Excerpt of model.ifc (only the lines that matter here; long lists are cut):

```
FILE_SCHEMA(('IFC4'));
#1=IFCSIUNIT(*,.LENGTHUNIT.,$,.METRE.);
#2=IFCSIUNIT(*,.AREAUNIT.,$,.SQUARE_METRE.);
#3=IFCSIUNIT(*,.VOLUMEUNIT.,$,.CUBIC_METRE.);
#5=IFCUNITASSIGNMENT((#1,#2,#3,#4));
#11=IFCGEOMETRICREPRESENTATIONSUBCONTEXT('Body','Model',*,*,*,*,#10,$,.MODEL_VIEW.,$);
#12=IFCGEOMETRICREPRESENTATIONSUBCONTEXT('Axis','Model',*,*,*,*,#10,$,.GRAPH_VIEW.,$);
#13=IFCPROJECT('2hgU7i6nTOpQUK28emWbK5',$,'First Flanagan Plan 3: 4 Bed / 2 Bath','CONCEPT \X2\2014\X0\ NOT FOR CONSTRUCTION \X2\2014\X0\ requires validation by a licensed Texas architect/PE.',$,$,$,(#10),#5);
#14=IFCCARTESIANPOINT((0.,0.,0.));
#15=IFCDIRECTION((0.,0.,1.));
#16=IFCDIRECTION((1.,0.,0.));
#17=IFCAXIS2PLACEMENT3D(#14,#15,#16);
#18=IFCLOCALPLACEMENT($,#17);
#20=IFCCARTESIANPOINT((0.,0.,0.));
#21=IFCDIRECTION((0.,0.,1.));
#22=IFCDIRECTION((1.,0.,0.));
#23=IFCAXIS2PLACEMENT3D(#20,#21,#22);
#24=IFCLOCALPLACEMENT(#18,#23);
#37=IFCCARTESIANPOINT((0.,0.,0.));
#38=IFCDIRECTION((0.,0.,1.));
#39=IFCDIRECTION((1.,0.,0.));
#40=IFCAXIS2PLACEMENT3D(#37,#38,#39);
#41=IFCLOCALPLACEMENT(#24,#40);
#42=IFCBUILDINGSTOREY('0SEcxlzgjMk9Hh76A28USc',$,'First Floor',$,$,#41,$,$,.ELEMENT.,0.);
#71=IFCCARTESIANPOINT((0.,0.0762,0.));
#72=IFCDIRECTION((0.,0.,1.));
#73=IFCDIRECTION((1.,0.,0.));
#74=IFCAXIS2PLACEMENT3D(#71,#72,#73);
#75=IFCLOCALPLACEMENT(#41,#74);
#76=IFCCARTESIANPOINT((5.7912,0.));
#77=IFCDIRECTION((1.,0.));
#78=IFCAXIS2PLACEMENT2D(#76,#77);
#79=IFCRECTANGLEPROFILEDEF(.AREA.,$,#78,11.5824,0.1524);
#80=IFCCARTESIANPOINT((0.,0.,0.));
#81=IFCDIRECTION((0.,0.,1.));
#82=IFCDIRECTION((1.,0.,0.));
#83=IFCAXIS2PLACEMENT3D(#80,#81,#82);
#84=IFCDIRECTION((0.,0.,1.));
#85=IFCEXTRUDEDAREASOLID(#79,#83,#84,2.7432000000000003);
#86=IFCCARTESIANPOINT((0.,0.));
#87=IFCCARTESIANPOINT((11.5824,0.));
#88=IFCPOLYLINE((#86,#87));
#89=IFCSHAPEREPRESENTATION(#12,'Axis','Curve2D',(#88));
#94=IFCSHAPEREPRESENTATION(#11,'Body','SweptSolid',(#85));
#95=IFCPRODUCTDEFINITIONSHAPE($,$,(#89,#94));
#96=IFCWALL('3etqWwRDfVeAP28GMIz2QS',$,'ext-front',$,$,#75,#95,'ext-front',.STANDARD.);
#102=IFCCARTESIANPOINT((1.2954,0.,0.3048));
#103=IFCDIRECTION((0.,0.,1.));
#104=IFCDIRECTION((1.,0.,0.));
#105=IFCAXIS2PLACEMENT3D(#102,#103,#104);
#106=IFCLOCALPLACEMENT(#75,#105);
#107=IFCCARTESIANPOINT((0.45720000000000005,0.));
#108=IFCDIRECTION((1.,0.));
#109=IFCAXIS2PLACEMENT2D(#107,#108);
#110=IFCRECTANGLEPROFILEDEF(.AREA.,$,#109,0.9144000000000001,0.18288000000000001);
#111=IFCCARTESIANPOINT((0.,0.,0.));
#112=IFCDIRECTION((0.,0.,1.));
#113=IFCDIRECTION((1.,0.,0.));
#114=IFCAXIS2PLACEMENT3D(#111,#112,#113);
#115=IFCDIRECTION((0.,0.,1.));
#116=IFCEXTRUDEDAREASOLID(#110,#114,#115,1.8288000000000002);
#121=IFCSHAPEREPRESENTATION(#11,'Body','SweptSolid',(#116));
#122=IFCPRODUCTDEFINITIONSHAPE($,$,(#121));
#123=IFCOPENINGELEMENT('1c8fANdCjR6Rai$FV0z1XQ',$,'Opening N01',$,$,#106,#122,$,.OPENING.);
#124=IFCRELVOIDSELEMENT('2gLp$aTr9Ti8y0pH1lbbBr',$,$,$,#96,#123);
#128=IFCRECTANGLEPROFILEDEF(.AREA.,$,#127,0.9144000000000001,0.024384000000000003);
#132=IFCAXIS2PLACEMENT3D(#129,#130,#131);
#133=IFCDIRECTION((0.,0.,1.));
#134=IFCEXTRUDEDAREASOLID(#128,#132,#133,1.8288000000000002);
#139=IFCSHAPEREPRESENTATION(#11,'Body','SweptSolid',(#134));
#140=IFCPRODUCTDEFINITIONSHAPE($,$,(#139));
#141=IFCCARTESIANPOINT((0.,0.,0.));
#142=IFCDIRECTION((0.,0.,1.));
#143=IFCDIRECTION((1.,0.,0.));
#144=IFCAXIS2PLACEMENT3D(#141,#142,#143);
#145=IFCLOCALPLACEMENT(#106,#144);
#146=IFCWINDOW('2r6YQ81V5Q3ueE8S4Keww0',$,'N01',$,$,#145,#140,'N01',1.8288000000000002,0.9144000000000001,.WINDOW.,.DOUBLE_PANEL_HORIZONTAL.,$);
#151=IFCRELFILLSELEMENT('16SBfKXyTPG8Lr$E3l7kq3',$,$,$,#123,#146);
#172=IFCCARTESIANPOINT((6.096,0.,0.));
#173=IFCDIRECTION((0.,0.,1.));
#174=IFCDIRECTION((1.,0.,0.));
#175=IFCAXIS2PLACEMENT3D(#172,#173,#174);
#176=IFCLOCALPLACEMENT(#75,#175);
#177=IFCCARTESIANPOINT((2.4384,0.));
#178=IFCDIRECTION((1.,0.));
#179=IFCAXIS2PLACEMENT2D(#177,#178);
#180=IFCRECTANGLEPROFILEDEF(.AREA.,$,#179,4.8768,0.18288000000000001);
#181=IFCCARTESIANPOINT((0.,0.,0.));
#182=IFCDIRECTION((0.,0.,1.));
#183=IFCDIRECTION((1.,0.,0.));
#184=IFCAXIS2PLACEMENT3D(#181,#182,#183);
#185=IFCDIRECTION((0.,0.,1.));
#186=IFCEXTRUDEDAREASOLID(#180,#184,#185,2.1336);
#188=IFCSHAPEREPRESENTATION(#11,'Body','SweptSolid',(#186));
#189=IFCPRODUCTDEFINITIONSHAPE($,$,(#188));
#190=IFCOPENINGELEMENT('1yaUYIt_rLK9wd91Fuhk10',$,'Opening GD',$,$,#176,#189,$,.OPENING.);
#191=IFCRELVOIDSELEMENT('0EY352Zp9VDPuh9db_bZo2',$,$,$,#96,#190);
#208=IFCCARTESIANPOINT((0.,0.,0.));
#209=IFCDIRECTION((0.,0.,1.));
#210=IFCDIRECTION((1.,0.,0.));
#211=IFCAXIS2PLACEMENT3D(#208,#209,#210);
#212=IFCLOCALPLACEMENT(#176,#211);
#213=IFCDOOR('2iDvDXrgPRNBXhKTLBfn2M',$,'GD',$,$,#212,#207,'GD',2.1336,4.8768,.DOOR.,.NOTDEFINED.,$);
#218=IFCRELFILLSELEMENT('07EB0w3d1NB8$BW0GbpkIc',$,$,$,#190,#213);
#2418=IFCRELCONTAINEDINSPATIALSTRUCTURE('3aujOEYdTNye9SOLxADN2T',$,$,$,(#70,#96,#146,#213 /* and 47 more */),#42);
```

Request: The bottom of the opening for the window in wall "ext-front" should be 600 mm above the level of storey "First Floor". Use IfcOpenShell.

```python
import numpy as np
import ifcopenshell
import ifcopenshell.api.geometry
import ifcopenshell.geom
import ifcopenshell.util.element
import ifcopenshell.util.placement
import ifcopenshell.util.shape
import ifcopenshell.util.unit

model = ifcopenshell.open("model.ifc")
unit_scale = ifcopenshell.util.unit.calculate_unit_scale(model)

window = model.by_guid("2r6YQ81V5Q3ueE8S4Keww0")
opening = window.FillsVoids[0].RelatingOpeningElement
storey = ifcopenshell.util.element.get_container(window, ifc_class="IfcBuildingStorey")
level = ifcopenshell.util.placement.get_local_placement(storey.ObjectPlacement)[2, 3]

# The opening's origin need not be at the sill, so measure its lowest point.
shape = ifcopenshell.geom.create_shape(ifcopenshell.geom.settings(), opening)
bottom = ifcopenshell.util.shape.get_shape_bottom_elevation(shape, shape.geometry) / unit_scale
dz = level + 0.6 / unit_scale - bottom

shift = np.array([0.0, 0.0, dz])
# The window is placed relative to its opening, so it follows when the opening moves.
matrix = ifcopenshell.util.placement.get_local_placement(opening.ObjectPlacement)
matrix[:3, 3] += shift
ifcopenshell.api.geometry.edit_object_placement(
    model, product=opening, matrix=matrix, is_si=False, should_transform_children=True
)

print(f"moved by {dz * unit_scale:+.3f} m")

model.write("model_rev.ifc")
```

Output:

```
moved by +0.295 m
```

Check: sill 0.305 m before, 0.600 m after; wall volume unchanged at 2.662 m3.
